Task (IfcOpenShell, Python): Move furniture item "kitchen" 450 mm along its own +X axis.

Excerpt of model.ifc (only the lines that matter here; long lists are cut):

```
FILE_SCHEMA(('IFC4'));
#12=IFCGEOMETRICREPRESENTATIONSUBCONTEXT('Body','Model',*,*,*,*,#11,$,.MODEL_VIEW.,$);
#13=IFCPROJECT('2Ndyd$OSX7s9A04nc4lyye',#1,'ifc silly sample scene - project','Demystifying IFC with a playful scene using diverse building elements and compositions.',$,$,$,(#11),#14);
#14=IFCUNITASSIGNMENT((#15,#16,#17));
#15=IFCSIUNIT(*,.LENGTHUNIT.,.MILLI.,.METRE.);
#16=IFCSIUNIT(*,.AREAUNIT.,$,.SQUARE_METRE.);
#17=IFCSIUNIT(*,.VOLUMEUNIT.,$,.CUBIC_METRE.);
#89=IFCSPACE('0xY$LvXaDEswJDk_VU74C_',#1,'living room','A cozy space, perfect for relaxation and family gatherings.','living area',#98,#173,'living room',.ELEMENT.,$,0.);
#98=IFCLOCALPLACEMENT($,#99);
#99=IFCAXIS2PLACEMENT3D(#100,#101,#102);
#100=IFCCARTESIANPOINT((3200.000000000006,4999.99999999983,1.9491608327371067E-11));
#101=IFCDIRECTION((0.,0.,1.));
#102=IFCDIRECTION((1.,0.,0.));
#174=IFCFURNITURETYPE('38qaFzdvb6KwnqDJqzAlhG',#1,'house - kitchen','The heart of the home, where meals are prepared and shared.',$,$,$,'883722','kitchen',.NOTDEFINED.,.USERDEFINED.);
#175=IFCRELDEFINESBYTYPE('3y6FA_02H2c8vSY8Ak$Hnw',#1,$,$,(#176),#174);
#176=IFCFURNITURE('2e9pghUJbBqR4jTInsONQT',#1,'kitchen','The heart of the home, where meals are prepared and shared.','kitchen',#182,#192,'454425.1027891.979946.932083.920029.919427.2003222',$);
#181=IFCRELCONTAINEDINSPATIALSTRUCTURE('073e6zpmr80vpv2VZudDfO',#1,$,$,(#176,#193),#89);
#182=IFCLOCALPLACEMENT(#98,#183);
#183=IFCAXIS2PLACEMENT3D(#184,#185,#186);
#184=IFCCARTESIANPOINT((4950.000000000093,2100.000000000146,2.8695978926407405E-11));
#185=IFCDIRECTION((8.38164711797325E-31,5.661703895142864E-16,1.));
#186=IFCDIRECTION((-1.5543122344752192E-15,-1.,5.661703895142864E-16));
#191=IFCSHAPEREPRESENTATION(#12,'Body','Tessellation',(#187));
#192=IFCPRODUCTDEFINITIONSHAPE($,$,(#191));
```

```python
import ifcopenshell
import ifcopenshell.api.geometry
import ifcopenshell.util.placement
import ifcopenshell.util.unit

model = ifcopenshell.open("model.ifc")
unit_scale = ifcopenshell.util.unit.calculate_unit_scale(model)

item = model.by_guid("2e9pghUJbBqR4jTInsONQT")
matrix = ifcopenshell.util.placement.get_local_placement(item.ObjectPlacement)
matrix[:3, 3] += matrix[:3, 0] * 0.45 / unit_scale
ifcopenshell.api.geometry.edit_object_placement(model, product=item, matrix=matrix, is_si=False)

print(ifcopenshell.util.placement.get_local_placement(item.ObjectPlacement).round(3) + 0.0)

model.write("model_edited.ifc")
```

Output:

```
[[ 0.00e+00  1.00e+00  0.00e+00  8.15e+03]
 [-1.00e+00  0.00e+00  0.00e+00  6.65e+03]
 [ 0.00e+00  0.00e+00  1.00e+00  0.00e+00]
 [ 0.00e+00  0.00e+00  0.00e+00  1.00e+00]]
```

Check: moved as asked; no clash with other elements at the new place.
